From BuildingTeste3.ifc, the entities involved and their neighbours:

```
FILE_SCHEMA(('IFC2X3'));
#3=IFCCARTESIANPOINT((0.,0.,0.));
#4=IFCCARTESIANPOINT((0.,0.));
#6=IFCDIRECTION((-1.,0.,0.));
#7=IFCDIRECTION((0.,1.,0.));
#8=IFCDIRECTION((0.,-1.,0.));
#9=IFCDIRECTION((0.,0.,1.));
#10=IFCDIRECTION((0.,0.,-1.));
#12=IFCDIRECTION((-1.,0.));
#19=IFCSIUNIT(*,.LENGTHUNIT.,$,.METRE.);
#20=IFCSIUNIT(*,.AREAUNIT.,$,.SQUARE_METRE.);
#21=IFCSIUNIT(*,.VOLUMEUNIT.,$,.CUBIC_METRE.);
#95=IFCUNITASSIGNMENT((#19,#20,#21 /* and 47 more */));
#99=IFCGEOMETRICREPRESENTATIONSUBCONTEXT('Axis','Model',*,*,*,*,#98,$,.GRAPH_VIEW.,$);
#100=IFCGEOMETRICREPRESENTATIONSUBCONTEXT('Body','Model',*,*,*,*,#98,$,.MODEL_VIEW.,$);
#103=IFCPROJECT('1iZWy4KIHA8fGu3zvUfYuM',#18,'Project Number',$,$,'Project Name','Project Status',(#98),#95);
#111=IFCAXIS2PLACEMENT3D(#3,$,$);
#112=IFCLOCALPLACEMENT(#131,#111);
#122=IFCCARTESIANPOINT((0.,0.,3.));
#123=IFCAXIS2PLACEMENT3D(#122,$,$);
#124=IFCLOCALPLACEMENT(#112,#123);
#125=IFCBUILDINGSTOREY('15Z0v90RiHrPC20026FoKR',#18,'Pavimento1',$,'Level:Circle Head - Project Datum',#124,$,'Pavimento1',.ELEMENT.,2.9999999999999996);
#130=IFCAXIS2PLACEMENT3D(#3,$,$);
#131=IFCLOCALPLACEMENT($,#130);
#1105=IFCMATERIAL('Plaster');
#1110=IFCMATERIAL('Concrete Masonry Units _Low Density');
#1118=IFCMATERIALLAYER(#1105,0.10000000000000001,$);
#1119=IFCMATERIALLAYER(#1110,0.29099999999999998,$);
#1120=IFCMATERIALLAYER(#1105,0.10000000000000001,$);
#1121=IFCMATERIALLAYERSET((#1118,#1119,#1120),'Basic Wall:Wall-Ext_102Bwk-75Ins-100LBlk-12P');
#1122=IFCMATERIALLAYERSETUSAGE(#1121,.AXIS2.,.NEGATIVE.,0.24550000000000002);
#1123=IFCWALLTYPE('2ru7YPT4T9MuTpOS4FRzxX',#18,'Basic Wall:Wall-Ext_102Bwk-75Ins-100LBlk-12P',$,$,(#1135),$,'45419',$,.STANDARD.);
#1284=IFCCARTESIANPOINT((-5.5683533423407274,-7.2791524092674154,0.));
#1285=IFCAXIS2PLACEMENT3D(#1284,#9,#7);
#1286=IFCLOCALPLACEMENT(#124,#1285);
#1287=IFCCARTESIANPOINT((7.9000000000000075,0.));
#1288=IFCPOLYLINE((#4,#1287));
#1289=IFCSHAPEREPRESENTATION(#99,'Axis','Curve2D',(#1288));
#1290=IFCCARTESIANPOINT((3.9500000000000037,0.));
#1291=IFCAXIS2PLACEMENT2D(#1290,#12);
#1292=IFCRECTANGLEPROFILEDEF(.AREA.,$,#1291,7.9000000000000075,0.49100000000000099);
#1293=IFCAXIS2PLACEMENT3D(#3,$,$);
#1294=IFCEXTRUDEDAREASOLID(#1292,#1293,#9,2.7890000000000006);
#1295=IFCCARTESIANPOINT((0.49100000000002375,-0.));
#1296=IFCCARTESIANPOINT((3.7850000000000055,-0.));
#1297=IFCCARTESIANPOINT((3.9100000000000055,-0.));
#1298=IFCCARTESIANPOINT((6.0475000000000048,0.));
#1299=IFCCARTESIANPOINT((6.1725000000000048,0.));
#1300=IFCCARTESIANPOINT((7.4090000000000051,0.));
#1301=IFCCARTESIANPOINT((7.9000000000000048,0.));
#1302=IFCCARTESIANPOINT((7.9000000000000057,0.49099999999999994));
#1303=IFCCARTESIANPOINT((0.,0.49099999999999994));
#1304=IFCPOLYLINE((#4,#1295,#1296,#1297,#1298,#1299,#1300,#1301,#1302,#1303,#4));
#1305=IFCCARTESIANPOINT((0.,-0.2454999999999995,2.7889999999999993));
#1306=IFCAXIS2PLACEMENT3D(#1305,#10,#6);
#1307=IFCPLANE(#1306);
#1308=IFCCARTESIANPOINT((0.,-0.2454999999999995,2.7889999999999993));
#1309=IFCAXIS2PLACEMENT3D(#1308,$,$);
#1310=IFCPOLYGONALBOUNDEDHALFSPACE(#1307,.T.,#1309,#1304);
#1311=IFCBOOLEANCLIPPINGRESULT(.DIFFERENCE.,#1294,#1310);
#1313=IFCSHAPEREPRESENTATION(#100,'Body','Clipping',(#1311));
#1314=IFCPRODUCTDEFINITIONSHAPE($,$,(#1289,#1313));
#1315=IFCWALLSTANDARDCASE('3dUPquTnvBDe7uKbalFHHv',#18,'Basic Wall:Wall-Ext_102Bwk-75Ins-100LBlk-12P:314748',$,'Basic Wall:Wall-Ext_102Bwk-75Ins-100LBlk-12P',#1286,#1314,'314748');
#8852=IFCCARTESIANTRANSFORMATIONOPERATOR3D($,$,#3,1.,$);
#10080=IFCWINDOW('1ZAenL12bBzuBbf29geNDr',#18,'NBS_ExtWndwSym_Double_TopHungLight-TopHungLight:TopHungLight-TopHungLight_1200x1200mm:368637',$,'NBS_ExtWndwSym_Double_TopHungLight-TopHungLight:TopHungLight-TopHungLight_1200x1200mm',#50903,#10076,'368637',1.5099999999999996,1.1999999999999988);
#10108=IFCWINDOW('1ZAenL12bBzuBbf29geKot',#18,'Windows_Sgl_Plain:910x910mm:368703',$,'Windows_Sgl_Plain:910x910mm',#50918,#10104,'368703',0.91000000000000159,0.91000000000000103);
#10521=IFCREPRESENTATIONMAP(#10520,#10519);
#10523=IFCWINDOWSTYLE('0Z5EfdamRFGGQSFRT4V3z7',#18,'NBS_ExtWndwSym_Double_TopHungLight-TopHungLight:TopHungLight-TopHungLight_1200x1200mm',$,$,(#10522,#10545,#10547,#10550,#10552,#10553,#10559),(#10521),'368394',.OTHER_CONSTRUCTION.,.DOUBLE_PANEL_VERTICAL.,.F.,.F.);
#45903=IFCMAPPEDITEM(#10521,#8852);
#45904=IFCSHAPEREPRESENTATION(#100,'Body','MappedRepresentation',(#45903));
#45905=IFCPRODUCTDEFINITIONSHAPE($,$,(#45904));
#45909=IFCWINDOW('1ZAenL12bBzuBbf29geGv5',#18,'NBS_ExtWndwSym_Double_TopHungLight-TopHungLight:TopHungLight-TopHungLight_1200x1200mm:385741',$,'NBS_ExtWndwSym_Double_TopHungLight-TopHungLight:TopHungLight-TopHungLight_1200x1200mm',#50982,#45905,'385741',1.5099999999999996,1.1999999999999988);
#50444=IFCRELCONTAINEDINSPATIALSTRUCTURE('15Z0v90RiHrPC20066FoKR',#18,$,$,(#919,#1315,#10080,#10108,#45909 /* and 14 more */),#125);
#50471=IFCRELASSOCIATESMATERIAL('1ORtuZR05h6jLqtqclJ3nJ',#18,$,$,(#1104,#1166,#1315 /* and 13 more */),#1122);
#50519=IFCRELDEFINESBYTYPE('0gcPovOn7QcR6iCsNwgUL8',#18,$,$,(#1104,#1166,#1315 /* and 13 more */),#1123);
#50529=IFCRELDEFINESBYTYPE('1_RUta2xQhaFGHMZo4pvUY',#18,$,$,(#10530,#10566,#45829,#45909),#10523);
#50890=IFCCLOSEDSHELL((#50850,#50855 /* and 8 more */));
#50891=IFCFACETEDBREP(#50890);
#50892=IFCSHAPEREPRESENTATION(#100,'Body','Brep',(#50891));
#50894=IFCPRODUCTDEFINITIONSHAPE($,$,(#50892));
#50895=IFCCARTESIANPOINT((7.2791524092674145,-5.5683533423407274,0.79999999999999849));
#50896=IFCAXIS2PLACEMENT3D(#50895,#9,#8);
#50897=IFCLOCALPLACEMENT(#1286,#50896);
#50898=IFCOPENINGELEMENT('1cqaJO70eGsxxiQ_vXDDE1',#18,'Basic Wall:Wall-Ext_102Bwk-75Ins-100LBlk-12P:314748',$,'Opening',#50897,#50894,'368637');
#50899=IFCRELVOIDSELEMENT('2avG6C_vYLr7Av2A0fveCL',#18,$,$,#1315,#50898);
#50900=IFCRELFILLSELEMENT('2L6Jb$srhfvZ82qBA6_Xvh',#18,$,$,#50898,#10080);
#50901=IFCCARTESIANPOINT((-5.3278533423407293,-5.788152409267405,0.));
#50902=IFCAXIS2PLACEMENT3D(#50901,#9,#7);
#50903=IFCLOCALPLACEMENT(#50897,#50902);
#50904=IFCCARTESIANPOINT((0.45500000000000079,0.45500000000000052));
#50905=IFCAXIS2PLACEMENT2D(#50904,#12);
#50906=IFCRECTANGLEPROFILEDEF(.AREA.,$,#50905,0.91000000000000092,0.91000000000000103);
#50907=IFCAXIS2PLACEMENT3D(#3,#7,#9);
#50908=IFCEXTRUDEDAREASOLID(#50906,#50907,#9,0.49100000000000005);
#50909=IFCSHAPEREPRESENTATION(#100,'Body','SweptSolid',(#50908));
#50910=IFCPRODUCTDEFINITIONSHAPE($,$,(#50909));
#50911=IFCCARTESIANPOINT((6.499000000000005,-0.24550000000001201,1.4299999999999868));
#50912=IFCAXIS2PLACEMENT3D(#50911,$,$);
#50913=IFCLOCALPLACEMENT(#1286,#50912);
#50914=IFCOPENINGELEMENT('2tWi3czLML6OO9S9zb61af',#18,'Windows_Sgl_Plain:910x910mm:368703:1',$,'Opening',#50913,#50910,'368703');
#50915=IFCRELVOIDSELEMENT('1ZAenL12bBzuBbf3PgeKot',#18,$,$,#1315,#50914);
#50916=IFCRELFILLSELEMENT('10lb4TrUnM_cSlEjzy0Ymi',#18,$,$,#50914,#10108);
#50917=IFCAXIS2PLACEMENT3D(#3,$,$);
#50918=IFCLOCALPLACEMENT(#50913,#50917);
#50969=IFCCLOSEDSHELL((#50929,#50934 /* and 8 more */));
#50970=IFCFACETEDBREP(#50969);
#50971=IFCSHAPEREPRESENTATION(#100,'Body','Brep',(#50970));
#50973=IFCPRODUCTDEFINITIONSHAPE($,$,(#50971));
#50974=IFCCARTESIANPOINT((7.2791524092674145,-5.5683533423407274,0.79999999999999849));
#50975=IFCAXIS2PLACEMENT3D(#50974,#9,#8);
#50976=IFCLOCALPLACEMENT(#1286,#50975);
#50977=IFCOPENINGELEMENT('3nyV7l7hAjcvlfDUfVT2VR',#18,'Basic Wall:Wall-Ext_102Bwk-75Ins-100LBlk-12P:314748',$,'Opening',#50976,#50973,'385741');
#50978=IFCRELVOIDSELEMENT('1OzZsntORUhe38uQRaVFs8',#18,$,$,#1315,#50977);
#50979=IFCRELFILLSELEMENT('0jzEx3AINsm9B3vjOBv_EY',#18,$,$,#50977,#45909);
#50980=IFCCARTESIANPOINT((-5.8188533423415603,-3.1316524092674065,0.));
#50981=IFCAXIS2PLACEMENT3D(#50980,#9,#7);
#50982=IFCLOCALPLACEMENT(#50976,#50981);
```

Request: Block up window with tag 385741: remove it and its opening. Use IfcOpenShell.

```python
import ifcopenshell
import ifcopenshell.api.feature
import ifcopenshell.api.root
import ifcopenshell.geom
import ifcopenshell.util.shape

model = ifcopenshell.open("BuildingTeste3.ifc")
settings = ifcopenshell.geom.settings()


def volume(element):
    """Net volume in cubic metres, openings subtracted."""
    shape = ifcopenshell.geom.create_shape(settings, element)
    return ifcopenshell.util.shape.get_volume(shape.geometry)


window = model.by_guid("1ZAenL12bBzuBbf29geGv5")
opening = window.FillsVoids[0].RelatingOpeningElement
wall = opening.VoidsElements[0].RelatingBuildingElement
before = volume(wall)

ifcopenshell.api.root.remove_product(model, product=window)
ifcopenshell.api.feature.remove_feature(model, feature=opening)

after = volume(wall)

print(f"wall volume {before:.3f} -> {after:.3f} m3")

model.write("BuildingTeste3_updated.ifc")
```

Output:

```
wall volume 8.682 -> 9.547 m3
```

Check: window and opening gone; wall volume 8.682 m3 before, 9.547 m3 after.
